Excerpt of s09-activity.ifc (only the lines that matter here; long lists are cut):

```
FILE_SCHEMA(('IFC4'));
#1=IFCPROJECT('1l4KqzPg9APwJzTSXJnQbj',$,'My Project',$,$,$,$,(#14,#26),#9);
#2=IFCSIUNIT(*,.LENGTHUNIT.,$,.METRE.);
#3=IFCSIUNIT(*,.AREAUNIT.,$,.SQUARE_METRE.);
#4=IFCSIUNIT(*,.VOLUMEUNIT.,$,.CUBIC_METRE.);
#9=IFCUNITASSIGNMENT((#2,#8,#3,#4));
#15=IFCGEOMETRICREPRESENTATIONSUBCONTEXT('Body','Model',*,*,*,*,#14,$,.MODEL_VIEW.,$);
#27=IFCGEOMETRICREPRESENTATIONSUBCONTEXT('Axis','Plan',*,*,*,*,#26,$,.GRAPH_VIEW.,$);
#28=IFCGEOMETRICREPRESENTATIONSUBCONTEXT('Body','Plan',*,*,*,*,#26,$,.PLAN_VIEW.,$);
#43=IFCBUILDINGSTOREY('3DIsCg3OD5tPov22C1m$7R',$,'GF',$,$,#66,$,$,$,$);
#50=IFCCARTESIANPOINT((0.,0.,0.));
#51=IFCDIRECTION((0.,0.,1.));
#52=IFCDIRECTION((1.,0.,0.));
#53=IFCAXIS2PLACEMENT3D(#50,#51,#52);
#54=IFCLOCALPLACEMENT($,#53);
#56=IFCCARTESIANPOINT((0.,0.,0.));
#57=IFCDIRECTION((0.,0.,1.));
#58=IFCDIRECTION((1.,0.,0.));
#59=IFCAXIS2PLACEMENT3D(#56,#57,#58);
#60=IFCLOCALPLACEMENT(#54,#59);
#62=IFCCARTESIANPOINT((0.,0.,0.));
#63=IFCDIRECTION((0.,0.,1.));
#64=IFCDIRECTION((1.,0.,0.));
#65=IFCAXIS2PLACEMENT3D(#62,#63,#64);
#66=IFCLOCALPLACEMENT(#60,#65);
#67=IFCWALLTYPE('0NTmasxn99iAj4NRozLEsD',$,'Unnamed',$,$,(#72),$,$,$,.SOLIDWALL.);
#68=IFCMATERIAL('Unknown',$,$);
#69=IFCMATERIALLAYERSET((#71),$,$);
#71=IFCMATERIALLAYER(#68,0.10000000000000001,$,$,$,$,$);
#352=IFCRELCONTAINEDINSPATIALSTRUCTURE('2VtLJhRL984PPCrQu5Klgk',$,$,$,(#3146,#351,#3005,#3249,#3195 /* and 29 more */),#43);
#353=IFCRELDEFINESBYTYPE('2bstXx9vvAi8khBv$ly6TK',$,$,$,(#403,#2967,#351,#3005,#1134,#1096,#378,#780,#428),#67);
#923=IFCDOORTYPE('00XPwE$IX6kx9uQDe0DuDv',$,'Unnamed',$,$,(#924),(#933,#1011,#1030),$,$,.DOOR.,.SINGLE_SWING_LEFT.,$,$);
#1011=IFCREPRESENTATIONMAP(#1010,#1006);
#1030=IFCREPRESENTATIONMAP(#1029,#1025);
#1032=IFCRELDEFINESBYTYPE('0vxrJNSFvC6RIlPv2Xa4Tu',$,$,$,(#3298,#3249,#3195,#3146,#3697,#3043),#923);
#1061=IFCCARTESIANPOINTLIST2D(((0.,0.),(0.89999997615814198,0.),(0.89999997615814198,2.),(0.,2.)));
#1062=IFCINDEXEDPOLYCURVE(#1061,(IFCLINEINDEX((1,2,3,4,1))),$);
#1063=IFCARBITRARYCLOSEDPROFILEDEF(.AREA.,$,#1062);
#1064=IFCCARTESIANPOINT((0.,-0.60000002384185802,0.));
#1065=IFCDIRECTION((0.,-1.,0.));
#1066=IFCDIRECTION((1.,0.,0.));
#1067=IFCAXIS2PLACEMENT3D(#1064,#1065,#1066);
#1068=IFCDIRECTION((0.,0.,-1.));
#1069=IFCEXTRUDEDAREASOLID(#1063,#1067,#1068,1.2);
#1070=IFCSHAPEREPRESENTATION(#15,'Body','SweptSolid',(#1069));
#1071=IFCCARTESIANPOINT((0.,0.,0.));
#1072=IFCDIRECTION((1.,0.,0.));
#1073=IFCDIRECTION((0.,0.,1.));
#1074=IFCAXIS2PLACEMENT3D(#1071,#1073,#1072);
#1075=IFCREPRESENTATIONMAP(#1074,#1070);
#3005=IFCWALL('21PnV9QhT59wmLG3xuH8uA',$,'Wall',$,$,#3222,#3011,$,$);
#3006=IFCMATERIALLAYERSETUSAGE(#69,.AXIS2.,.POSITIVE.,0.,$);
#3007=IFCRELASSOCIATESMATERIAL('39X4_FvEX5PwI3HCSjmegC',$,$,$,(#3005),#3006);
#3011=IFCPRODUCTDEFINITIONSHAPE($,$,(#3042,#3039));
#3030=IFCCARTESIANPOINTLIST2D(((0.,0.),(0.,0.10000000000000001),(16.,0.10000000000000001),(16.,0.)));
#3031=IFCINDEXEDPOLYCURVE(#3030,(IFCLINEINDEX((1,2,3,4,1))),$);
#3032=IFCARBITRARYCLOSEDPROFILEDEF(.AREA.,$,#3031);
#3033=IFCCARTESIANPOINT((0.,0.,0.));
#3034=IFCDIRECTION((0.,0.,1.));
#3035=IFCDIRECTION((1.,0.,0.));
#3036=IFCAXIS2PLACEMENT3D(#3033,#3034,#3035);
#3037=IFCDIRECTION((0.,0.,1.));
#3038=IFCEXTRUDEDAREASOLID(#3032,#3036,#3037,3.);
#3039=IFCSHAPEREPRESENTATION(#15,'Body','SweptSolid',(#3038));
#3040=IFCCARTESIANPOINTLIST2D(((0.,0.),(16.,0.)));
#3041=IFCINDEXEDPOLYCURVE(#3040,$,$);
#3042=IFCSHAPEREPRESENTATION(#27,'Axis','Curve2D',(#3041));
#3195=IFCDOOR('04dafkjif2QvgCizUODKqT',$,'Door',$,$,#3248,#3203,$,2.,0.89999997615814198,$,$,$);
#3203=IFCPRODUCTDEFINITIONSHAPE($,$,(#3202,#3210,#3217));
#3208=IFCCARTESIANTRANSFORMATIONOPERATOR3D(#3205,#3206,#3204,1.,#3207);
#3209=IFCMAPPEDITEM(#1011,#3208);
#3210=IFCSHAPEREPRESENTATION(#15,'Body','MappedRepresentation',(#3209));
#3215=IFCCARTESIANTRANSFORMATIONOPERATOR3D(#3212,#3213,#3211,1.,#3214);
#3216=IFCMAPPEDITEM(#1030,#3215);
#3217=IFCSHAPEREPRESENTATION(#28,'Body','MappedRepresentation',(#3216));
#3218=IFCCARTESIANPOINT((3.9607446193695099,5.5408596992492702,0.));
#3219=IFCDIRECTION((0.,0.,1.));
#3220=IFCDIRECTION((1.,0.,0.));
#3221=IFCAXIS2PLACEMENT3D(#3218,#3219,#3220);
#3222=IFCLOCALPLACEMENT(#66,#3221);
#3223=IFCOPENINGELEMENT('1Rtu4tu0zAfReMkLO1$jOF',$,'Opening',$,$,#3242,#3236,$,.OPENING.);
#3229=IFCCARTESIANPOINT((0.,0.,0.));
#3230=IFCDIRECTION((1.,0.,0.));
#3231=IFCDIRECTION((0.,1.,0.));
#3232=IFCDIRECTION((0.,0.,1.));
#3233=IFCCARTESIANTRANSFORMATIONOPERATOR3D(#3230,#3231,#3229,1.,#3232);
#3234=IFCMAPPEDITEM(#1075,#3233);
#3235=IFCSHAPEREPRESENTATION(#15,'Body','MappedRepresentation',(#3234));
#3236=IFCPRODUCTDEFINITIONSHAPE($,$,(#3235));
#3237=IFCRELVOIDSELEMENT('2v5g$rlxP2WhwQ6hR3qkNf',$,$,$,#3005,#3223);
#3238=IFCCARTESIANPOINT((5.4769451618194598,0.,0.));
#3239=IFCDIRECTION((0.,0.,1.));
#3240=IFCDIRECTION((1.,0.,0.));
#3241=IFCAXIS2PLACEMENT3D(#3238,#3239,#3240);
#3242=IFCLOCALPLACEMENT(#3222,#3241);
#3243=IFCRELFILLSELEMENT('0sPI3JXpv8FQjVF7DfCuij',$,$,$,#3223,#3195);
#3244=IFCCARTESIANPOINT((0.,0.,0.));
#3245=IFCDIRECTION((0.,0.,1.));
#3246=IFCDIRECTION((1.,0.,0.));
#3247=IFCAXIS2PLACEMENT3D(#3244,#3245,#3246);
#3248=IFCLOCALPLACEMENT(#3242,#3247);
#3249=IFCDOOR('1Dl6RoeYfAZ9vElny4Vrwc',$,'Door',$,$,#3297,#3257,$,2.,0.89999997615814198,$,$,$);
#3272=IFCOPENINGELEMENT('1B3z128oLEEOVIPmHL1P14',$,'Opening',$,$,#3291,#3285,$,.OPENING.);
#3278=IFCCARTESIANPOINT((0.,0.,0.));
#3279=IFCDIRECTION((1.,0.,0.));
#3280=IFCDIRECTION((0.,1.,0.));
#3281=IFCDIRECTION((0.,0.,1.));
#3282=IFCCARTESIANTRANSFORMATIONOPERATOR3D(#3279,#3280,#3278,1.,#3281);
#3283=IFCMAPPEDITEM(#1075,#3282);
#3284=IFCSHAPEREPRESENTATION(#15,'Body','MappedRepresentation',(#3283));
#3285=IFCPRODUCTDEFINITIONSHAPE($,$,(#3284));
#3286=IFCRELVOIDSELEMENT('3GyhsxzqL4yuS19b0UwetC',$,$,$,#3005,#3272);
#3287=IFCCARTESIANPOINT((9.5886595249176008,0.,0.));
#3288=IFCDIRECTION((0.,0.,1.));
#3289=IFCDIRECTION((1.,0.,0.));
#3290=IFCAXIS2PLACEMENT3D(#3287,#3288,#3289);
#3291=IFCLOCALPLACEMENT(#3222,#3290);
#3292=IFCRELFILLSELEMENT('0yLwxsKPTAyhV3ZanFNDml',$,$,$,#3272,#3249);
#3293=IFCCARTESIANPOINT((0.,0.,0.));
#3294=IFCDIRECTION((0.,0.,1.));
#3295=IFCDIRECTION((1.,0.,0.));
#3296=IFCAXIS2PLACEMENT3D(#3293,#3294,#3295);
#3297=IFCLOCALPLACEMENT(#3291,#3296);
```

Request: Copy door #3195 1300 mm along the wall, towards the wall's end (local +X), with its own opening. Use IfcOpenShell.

```python
import ifcopenshell
import ifcopenshell.api.feature
import ifcopenshell.api.geometry
import ifcopenshell.api.root
import ifcopenshell.geom
import ifcopenshell.util.element
import ifcopenshell.util.placement
import ifcopenshell.util.shape
import ifcopenshell.util.unit

model = ifcopenshell.open("s09-activity.ifc")
unit_scale = ifcopenshell.util.unit.calculate_unit_scale(model)
settings = ifcopenshell.geom.settings()


def volume(element):
    """Net volume in cubic metres, openings subtracted."""
    shape = ifcopenshell.geom.create_shape(settings, element)
    return ifcopenshell.util.shape.get_volume(shape.geometry)


door = model.by_guid("04dafkjif2QvgCizUODKqT")
opening = door.FillsVoids[0].RelatingOpeningElement
wall = opening.VoidsElements[0].RelatingBuildingElement
before = volume(wall)
shift = ifcopenshell.util.placement.get_local_placement(wall.ObjectPlacement)[:3, 0] * 1.3 / unit_scale

# copy_class copies the void relationship, type, container and properties, but no geometry.
new_opening = ifcopenshell.api.root.copy_class(model, product=opening)
new_opening.Representation = ifcopenshell.util.element.copy_deep(
    model, opening.Representation, exclude=["IfcGeometricRepresentationContext", "IfcRepresentationMap"]
)
new_door = ifcopenshell.api.root.copy_class(model, product=door)
new_door.Representation = ifcopenshell.util.element.copy_deep(
    model, door.Representation, exclude=["IfcGeometricRepresentationContext", "IfcRepresentationMap"]
)
ifcopenshell.api.feature.add_filling(model, opening=new_opening, element=new_door)

for old, new in ((opening, new_opening), (door, new_door)):
    matrix = ifcopenshell.util.placement.get_local_placement(old.ObjectPlacement)
    matrix[:3, 3] += shift
    ifcopenshell.api.geometry.edit_object_placement(model, product=new, matrix=matrix, is_si=False)

after = volume(wall)

print(f"wall volume {before:.3f} -> {after:.3f} m3")

model.write("s09-activity-out.ifc")
```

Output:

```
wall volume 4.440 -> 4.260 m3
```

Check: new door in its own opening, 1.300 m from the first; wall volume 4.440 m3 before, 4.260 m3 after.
